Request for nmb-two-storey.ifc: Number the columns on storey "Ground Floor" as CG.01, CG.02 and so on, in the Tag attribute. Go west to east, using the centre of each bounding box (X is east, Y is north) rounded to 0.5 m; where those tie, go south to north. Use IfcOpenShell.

First a look at what the model holds.

```python
import ifcopenshell
import ifcopenshell.util.element
import ifcopenshell.util.placement

model = ifcopenshell.open("nmb-two-storey.ifc")
print(model.schema)
storey = next(s for s in model.by_type("IfcBuildingStorey") if s.Name == "Ground Floor")
columns = [e for e in ifcopenshell.util.element.get_decomposition(storey) if e.is_a("IfcColumn")]
for e in sorted(columns, key=lambda e: e.id()):
    origin = ifcopenshell.util.placement.get_local_placement(e.ObjectPlacement)[:3, 3]
    print(e.id(), e.Tag, e.Name, origin.round(2) + 0.0, sep=" | ")
```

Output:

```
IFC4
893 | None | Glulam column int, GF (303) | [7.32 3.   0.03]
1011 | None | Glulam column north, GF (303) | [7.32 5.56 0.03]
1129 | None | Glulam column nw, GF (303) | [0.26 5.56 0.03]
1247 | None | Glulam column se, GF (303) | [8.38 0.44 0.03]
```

```python
import ifcopenshell
import ifcopenshell.geom
import ifcopenshell.util.element
import ifcopenshell.util.shape

model = ifcopenshell.open("nmb-two-storey.ifc")
settings = ifcopenshell.geom.settings()
settings.set("use-world-coords", True)


def centre(element):
    shape = ifcopenshell.geom.create_shape(settings, element)
    return ifcopenshell.util.shape.get_bbox_centroid(shape.geometry)


storey = next(s for s in model.by_type("IfcBuildingStorey") if s.Name == "Ground Floor")
columns = [e for e in ifcopenshell.util.element.get_decomposition(storey) if e.is_a("IfcColumn")]

# Insertion points can sit at a corner or the storey origin, so sort by the geometry (in metres).
centres = {e: centre(e) for e in columns}
columns.sort(key=lambda e: (round(centres[e][0] / 0.5), centres[e][1]))

for i, e in enumerate(columns, start=1):
    number = f"CG.{i:02d}"
    e.Tag = number
    print(e.id(), number)

model.write("nmb-two-storey_v2.ifc")
```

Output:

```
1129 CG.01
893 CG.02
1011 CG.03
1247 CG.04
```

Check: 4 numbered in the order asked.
